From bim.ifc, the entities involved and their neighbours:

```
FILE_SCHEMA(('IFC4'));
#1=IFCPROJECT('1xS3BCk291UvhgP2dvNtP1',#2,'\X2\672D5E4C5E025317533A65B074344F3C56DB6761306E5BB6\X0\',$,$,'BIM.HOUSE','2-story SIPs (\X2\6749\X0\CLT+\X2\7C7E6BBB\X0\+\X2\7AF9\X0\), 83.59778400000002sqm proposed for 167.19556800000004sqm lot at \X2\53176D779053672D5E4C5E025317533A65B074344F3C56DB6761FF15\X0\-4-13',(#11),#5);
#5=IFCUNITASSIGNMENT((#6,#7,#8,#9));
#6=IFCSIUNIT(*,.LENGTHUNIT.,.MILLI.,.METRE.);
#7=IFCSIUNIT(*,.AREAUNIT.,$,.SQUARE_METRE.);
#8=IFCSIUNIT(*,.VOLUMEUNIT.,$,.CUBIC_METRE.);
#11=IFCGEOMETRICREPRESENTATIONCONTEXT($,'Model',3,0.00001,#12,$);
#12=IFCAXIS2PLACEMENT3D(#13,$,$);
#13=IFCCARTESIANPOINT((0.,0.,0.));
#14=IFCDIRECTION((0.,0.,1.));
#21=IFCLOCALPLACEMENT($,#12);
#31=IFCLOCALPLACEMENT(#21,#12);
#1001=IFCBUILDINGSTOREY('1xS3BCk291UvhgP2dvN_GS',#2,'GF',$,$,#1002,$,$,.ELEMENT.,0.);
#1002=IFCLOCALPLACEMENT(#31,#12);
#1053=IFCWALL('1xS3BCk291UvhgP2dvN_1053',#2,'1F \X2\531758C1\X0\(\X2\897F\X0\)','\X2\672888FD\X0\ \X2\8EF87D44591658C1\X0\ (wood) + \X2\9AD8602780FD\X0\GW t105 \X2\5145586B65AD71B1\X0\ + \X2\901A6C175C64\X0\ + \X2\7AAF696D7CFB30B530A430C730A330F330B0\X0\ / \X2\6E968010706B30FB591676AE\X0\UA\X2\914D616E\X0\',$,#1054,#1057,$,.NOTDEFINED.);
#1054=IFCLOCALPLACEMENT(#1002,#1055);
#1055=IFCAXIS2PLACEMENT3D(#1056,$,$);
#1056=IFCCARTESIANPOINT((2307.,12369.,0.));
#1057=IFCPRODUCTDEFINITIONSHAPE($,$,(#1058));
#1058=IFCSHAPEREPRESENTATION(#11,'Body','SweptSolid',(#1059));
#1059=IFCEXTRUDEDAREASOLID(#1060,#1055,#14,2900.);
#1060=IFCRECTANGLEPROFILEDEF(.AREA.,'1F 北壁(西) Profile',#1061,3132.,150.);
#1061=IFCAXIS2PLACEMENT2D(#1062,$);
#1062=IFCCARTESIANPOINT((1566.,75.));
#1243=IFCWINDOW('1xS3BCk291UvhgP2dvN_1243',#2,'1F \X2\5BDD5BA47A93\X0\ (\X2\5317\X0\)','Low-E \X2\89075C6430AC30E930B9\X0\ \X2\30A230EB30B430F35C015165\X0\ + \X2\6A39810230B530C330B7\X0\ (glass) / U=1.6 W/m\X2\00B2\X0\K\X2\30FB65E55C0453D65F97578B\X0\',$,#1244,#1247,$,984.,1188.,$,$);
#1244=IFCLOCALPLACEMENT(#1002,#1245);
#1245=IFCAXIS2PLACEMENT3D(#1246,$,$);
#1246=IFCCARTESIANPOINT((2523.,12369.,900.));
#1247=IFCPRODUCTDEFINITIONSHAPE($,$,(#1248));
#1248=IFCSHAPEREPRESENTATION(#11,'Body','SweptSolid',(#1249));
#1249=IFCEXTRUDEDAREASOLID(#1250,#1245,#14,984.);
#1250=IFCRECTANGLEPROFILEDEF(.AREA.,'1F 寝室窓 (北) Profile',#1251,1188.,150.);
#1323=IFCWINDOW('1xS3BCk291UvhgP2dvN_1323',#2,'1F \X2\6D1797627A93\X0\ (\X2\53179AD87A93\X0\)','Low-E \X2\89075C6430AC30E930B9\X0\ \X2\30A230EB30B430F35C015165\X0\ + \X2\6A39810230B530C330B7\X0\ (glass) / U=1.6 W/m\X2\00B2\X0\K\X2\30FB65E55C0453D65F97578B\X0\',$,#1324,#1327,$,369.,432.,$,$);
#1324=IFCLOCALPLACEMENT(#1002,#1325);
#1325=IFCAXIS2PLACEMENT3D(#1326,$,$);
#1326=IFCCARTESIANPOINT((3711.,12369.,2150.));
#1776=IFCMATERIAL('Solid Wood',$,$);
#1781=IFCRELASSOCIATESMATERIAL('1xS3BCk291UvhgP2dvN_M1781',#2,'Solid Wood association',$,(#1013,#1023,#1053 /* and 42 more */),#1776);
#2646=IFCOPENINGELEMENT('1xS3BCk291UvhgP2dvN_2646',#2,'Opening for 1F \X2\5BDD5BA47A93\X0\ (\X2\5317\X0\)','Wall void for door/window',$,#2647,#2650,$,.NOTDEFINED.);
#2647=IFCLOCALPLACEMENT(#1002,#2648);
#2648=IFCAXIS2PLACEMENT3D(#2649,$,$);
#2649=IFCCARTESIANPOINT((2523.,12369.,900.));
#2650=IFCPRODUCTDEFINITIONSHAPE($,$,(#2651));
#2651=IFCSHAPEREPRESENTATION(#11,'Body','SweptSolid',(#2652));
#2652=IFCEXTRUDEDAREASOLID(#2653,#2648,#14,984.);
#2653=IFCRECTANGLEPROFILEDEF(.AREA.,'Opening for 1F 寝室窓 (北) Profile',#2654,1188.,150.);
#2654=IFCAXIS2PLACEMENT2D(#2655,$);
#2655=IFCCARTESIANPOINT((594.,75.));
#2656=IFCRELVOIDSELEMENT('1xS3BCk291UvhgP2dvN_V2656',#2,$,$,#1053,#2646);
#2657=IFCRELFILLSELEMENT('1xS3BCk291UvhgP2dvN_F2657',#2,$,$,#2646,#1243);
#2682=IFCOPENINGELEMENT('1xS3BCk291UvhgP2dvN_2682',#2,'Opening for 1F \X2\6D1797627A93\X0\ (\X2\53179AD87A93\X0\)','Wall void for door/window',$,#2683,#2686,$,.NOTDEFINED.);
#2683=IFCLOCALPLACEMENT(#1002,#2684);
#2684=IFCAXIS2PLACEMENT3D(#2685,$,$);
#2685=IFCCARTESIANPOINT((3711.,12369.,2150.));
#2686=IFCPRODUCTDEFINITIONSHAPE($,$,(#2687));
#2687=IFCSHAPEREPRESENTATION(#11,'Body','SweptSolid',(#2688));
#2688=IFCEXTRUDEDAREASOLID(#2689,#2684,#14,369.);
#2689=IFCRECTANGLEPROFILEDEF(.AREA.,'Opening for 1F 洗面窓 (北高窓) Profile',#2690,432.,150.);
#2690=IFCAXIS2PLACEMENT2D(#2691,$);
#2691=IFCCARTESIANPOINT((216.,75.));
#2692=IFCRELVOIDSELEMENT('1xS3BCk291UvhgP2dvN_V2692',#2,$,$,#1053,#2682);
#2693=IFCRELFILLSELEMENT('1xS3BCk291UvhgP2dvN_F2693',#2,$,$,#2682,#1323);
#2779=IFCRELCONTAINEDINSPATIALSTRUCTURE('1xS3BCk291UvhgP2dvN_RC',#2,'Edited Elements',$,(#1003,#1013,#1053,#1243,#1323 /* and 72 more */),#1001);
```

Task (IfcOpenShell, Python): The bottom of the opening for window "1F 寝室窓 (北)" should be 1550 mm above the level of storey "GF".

```python
import numpy as np
import ifcopenshell
import ifcopenshell.api.geometry
import ifcopenshell.geom
import ifcopenshell.util.element
import ifcopenshell.util.placement
import ifcopenshell.util.shape
import ifcopenshell.util.unit

model = ifcopenshell.open("bim.ifc")
unit_scale = ifcopenshell.util.unit.calculate_unit_scale(model)

window = model.by_guid("1xS3BCk291UvhgP2dvN_1243")
opening = window.FillsVoids[0].RelatingOpeningElement
storey = ifcopenshell.util.element.get_container(window, ifc_class="IfcBuildingStorey")
level = ifcopenshell.util.placement.get_local_placement(storey.ObjectPlacement)[2, 3]

# The opening's origin need not be at the sill, so measure its lowest point.
shape = ifcopenshell.geom.create_shape(ifcopenshell.geom.settings(), opening)
bottom = ifcopenshell.util.shape.get_shape_bottom_elevation(shape, shape.geometry) / unit_scale
dz = level + 1.55 / unit_scale - bottom

shift = np.array([0.0, 0.0, dz])
# The window is not placed relative to its opening, so move both.
for product in (opening, window):
    matrix = ifcopenshell.util.placement.get_local_placement(product.ObjectPlacement)
    matrix[:3, 3] += shift
    ifcopenshell.api.geometry.edit_object_placement(model, product=product, matrix=matrix, is_si=False)

print(f"moved by {dz * unit_scale:+.3f} m")

model.write("bim-out.ifc")
```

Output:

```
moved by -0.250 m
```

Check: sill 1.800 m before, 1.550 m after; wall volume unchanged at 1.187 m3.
